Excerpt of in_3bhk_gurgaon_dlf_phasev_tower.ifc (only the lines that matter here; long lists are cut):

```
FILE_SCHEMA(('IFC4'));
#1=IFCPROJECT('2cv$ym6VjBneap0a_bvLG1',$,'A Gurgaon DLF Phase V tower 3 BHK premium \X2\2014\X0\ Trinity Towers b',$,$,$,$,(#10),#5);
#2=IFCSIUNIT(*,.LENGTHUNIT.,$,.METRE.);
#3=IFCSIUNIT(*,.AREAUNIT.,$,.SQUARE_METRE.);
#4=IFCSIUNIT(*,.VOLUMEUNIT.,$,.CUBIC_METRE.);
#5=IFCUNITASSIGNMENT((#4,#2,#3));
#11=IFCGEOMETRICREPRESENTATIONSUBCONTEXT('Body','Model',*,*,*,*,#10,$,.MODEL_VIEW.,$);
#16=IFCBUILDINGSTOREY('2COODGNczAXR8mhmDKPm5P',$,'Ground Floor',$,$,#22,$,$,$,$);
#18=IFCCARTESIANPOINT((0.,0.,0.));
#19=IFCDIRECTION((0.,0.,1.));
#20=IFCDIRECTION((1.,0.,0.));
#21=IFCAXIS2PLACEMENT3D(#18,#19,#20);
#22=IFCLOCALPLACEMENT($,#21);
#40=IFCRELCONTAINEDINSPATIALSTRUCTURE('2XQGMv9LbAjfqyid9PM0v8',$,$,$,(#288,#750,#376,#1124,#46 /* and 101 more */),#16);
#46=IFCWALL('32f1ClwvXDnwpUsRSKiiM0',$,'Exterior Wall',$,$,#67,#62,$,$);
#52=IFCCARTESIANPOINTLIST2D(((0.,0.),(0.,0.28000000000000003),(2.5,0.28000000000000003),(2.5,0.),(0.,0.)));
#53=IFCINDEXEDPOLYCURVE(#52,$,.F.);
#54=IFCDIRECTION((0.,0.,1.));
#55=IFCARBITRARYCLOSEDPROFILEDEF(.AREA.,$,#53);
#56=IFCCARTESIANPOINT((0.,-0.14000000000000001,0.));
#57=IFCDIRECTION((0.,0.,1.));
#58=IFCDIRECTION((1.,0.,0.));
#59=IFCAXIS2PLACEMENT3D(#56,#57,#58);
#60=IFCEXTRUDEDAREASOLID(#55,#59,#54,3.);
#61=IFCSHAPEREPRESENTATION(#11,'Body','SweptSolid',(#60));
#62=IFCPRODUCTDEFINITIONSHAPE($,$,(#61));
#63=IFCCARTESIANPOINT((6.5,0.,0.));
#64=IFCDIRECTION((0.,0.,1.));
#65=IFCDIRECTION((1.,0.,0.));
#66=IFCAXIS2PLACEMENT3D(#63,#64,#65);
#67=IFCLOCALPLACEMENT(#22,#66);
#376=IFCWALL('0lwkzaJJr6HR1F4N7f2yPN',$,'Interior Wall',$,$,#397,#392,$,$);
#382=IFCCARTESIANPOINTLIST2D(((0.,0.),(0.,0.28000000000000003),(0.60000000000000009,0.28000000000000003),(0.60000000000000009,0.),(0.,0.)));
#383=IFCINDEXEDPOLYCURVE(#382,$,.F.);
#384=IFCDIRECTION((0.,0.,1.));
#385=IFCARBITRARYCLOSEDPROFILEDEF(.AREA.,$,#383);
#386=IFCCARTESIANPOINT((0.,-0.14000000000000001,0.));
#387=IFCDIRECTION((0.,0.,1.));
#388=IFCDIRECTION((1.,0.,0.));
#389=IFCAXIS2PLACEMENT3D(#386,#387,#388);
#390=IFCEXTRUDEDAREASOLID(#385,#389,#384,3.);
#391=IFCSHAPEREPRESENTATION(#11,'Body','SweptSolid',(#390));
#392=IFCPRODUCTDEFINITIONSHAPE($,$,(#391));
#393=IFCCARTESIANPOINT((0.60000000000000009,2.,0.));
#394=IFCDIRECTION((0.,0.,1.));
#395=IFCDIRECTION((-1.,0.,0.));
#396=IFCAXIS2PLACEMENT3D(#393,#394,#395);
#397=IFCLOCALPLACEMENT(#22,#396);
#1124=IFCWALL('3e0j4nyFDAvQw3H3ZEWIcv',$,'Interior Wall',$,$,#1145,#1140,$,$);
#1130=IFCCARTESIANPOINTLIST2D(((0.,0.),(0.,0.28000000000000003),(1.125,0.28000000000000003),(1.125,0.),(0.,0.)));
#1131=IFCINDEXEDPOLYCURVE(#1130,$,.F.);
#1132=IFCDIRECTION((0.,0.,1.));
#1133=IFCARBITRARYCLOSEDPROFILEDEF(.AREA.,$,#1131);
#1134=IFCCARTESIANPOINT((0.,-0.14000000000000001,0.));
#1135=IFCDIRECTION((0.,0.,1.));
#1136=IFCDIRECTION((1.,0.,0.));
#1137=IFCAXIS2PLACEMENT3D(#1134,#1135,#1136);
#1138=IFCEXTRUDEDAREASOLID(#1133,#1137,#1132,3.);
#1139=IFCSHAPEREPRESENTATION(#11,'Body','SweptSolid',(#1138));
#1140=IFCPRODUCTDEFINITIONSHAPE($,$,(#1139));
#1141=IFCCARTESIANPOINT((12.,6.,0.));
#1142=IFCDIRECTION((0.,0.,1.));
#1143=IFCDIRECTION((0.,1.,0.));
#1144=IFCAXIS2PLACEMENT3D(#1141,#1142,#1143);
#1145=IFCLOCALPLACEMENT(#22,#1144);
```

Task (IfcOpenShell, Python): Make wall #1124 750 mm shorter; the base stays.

```python
import ifcopenshell
import ifcopenshell.geom
import ifcopenshell.util.representation
import ifcopenshell.util.shape
import ifcopenshell.util.unit

model = ifcopenshell.open("in_3bhk_gurgaon_dlf_phasev_tower.ifc")
unit_scale = ifcopenshell.util.unit.calculate_unit_scale(model)
settings = ifcopenshell.geom.settings()


def volume(element):
    """Net volume in cubic metres, openings subtracted."""
    shape = ifcopenshell.geom.create_shape(settings, element)
    return ifcopenshell.util.shape.get_volume(shape.geometry)


wall = model.by_guid("3e0j4nyFDAvQw3H3ZEWIcv")
before = volume(wall)

body = ifcopenshell.util.representation.get_representation(wall, "Model", "Body")
solid = body.Items[0]
old_height = solid.Depth
solid.Depth -= 0.75 / unit_scale
after = volume(wall)

print(f"height {old_height:g} -> {solid.Depth:g}, volume {before:.3f} -> {after:.3f} m3")

model.write("in_3bhk_gurgaon_dlf_phasev_tower_rev.ifc")
```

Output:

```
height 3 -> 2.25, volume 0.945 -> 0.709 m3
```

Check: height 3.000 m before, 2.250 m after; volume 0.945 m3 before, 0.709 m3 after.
